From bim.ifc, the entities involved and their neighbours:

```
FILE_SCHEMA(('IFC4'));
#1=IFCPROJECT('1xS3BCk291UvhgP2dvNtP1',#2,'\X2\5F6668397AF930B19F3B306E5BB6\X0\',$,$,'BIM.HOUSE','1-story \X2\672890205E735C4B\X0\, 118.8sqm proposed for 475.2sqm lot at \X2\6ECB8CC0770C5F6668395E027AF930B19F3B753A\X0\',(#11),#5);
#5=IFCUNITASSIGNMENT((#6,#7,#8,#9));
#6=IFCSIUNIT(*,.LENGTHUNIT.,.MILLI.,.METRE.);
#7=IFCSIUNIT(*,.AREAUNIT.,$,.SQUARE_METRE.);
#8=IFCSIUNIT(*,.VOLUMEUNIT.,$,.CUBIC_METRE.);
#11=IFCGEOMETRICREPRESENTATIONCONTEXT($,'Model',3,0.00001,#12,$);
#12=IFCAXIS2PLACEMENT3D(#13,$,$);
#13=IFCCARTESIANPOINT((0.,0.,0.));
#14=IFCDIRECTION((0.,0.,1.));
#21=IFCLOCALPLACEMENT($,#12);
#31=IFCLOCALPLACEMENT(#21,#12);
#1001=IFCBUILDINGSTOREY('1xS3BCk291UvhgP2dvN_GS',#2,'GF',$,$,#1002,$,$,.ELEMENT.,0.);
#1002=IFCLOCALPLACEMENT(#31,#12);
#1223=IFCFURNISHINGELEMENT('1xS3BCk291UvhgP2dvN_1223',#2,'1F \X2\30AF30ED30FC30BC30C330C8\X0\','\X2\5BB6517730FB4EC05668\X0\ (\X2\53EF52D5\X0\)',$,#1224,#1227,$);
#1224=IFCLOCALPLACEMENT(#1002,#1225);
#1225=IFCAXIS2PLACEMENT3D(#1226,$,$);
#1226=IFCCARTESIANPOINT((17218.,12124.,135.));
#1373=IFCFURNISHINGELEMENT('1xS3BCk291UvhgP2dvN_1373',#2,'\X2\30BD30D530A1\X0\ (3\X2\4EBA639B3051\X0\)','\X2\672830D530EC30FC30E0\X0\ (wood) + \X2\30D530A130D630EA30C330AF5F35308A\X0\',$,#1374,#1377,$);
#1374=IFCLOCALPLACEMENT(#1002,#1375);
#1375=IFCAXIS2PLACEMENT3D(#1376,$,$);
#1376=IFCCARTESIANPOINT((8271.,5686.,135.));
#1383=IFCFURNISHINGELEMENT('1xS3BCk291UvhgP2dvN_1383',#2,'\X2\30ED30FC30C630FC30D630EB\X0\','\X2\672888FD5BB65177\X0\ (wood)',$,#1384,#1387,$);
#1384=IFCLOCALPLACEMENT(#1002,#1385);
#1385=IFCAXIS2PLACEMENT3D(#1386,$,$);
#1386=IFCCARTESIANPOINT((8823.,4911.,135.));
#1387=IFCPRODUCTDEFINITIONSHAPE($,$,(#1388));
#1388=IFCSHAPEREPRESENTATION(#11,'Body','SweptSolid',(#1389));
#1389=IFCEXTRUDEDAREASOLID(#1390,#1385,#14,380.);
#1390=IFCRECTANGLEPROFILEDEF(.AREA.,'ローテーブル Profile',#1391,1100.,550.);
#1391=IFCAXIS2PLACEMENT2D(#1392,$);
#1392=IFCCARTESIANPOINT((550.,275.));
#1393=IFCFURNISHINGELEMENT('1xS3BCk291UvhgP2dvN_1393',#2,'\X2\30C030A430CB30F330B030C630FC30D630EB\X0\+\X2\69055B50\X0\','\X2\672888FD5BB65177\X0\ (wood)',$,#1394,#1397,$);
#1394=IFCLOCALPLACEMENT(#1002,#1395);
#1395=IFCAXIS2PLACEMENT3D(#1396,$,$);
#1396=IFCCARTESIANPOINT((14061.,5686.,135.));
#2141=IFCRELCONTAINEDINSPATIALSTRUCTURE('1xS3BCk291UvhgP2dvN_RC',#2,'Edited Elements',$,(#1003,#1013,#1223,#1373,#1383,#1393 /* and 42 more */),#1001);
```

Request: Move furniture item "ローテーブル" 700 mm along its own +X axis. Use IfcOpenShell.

```python
import ifcopenshell
import ifcopenshell.api.geometry
import ifcopenshell.util.placement
import ifcopenshell.util.unit

model = ifcopenshell.open("bim.ifc")
unit_scale = ifcopenshell.util.unit.calculate_unit_scale(model)

item = model.by_guid("1xS3BCk291UvhgP2dvN_1383")
matrix = ifcopenshell.util.placement.get_local_placement(item.ObjectPlacement)
matrix[:3, 3] += matrix[:3, 0] * 0.7 / unit_scale
ifcopenshell.api.geometry.edit_object_placement(model, product=item, matrix=matrix, is_si=False)

print(ifcopenshell.util.placement.get_local_placement(item.ObjectPlacement).round(3) + 0.0)

model.write("bim_updated.ifc")
```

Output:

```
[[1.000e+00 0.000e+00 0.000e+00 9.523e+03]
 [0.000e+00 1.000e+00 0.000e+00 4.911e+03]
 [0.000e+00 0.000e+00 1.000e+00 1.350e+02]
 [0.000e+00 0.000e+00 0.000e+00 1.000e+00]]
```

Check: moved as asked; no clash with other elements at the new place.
